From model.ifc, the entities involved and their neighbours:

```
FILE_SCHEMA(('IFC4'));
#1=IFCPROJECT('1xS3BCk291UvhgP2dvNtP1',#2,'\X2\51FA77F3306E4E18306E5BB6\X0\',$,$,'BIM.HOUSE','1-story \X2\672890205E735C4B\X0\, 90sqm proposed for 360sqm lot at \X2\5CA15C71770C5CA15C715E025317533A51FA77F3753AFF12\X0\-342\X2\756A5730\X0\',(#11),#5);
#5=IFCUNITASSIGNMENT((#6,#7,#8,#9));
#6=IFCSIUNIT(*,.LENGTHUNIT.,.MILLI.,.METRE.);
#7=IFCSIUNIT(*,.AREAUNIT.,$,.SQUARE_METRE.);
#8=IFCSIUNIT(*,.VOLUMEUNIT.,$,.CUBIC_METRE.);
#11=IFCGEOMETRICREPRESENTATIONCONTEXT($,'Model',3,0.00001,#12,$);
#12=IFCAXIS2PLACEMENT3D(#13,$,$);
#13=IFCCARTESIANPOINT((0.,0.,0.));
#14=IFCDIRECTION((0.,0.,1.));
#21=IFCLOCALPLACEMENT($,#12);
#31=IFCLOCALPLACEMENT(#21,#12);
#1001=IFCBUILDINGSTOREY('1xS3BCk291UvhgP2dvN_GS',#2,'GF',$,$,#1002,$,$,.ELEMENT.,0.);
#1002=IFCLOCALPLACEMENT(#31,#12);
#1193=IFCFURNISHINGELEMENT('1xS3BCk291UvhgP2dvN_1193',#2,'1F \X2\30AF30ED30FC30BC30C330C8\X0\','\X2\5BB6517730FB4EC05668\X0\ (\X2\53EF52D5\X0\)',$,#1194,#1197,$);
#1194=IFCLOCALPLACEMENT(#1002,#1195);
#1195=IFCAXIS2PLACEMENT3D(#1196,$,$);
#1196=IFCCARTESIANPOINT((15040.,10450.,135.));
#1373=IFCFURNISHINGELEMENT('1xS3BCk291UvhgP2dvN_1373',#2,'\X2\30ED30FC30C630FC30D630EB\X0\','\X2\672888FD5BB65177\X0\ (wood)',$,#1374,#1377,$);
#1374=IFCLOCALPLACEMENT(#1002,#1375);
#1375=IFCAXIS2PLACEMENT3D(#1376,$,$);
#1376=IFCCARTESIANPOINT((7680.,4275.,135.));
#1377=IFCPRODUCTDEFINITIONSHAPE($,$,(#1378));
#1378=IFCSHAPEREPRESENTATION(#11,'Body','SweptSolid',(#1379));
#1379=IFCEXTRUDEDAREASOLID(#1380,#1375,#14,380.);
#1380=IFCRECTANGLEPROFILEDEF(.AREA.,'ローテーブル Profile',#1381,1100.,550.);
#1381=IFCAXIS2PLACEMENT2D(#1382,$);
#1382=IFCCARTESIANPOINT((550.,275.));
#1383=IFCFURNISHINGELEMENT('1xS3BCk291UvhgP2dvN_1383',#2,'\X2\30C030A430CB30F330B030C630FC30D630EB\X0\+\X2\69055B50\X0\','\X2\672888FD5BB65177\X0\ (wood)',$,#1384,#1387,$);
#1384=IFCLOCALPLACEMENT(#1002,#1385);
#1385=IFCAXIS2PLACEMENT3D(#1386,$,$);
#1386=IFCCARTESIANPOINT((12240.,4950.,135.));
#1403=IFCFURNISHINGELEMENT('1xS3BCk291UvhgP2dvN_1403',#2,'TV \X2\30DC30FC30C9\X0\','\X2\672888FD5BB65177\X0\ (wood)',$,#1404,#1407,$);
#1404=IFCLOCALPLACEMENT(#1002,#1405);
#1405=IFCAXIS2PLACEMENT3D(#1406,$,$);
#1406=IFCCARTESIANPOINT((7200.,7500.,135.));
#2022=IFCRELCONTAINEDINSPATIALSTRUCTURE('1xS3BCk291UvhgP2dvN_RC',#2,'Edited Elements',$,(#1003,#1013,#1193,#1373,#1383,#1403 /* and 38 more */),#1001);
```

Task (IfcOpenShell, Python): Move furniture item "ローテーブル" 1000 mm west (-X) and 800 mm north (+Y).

```python
import ifcopenshell
import ifcopenshell.api.geometry
import ifcopenshell.util.placement
import ifcopenshell.util.unit

model = ifcopenshell.open("model.ifc")
unit_scale = ifcopenshell.util.unit.calculate_unit_scale(model)

item = model.by_guid("1xS3BCk291UvhgP2dvN_1373")
matrix = ifcopenshell.util.placement.get_local_placement(item.ObjectPlacement)
matrix[0, 3] -= 1 / unit_scale
matrix[1, 3] += 0.8 / unit_scale
ifcopenshell.api.geometry.edit_object_placement(model, product=item, matrix=matrix, is_si=False)

print(ifcopenshell.util.placement.get_local_placement(item.ObjectPlacement).round(3) + 0.0)

model.write("model_edited.ifc")
```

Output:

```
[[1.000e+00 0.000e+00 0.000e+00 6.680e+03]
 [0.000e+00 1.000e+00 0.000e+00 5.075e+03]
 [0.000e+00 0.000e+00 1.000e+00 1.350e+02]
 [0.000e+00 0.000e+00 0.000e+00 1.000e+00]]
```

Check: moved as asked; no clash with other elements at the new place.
